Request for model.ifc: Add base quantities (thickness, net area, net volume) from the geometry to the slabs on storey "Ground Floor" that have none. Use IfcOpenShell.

First a look at what the model holds.

```python
import ifcopenshell
import ifcopenshell.util.element
import ifcopenshell.util.unit

model = ifcopenshell.open("model.ifc")
print(model.schema)
for unit_type in ("LENGTHUNIT", "AREAUNIT", "VOLUMEUNIT"):
    print(unit_type, ifcopenshell.util.unit.calculate_unit_scale(model, unit_type))
storey = next(s for s in model.by_type("IfcBuildingStorey") if s.Name == "Ground Floor")
slabs = [e for e in ifcopenshell.util.element.get_decomposition(storey) if e.is_a("IfcSlab")]
for e in sorted(slabs, key=lambda e: e.id()):
    print(e.id(), e.is_a(), e.Name, list(ifcopenshell.util.element.get_psets(e, qtos_only=True)), sep=" | ")
```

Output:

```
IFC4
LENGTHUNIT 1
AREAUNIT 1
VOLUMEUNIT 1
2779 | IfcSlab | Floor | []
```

```python
import ifcopenshell
import ifcopenshell.api.pset
import ifcopenshell.geom
import ifcopenshell.util.element
import ifcopenshell.util.shape
import ifcopenshell.util.unit

model = ifcopenshell.open("model.ifc")
unit_scale = ifcopenshell.util.unit.calculate_unit_scale(model)
area_scale = ifcopenshell.util.unit.calculate_unit_scale(model, "AREAUNIT")
volume_scale = ifcopenshell.util.unit.calculate_unit_scale(model, "VOLUMEUNIT")
settings = ifcopenshell.geom.settings()

storey = next(s for s in model.by_type("IfcBuildingStorey") if s.Name == "Ground Floor")
slabs = [e for e in ifcopenshell.util.element.get_decomposition(storey) if e.is_a("IfcSlab")]

for e in sorted(slabs, key=lambda e: e.id()):
    if ifcopenshell.util.element.get_psets(e, qtos_only=True, should_inherit=False):
        continue
    # Geometry comes back in metres, in the element's own axes.
    shape = ifcopenshell.geom.create_shape(settings, e)
    values = {
        "Width": ifcopenshell.util.shape.get_z(shape.geometry) / unit_scale,
        "NetArea": ifcopenshell.util.shape.get_footprint_area(shape.geometry) / area_scale,
        "NetVolume": ifcopenshell.util.shape.get_volume(shape.geometry) / volume_scale,
    }
    qto = ifcopenshell.api.pset.add_qto(model, product=e, name="Qto_SlabBaseQuantities")
    ifcopenshell.api.pset.edit_qto(model, qto=qto, properties=values)
    print(e.id(), {k: round(v, 3) for k, v in values.items()})

model.write("model_updated.ifc")
```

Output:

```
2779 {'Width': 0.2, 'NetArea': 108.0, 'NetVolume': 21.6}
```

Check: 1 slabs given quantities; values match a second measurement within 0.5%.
